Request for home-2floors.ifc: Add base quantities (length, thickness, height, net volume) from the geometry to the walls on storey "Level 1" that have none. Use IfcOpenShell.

First a look at what the model holds.

```python
import ifcopenshell
import ifcopenshell.util.element
import ifcopenshell.util.unit

model = ifcopenshell.open("home-2floors.ifc")
print(model.schema)
for unit_type in ("LENGTHUNIT", "AREAUNIT", "VOLUMEUNIT"):
    print(unit_type, ifcopenshell.util.unit.calculate_unit_scale(model, unit_type))
storey = next(s for s in model.by_type("IfcBuildingStorey") if s.Name == "Level 1")
walls = [e for e in ifcopenshell.util.element.get_decomposition(storey) if e.is_a("IfcWall")]
for e in sorted(walls, key=lambda e: e.id()):
    print(e.id(), e.is_a(), e.Name, list(ifcopenshell.util.element.get_psets(e, qtos_only=True)), sep=" | ")
```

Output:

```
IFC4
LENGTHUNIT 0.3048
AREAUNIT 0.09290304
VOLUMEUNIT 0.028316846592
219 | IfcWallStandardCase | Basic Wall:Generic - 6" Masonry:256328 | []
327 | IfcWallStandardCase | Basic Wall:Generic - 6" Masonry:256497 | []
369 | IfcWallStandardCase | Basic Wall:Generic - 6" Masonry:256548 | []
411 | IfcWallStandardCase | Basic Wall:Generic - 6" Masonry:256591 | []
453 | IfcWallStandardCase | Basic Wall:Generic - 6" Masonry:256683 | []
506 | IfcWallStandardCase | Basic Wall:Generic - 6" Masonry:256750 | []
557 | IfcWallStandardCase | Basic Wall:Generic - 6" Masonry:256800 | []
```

```python
import ifcopenshell
import ifcopenshell.api.pset
import ifcopenshell.geom
import ifcopenshell.util.element
import ifcopenshell.util.shape
import ifcopenshell.util.unit

model = ifcopenshell.open("home-2floors.ifc")
unit_scale = ifcopenshell.util.unit.calculate_unit_scale(model)
volume_scale = ifcopenshell.util.unit.calculate_unit_scale(model, "VOLUMEUNIT")
settings = ifcopenshell.geom.settings()

storey = next(s for s in model.by_type("IfcBuildingStorey") if s.Name == "Level 1")
walls = [e for e in ifcopenshell.util.element.get_decomposition(storey) if e.is_a("IfcWall")]

for e in sorted(walls, key=lambda e: e.id()):
    if ifcopenshell.util.element.get_psets(e, qtos_only=True, should_inherit=False):
        continue
    # Geometry comes back in metres, in the element's own axes.
    shape = ifcopenshell.geom.create_shape(settings, e)
    values = {
        "Length": ifcopenshell.util.shape.get_x(shape.geometry) / unit_scale,
        "Width": ifcopenshell.util.shape.get_y(shape.geometry) / unit_scale,
        "Height": ifcopenshell.util.shape.get_z(shape.geometry) / unit_scale,
        "NetVolume": ifcopenshell.util.shape.get_volume(shape.geometry) / volume_scale,
    }
    qto = ifcopenshell.api.pset.add_qto(model, product=e, name="Qto_WallBaseQuantities")
    ifcopenshell.api.pset.edit_qto(model, qto=qto, properties=values)
    print(e.id(), {k: round(v, 3) for k, v in values.items()})

model.write("home-2floors_rev.ifc")
```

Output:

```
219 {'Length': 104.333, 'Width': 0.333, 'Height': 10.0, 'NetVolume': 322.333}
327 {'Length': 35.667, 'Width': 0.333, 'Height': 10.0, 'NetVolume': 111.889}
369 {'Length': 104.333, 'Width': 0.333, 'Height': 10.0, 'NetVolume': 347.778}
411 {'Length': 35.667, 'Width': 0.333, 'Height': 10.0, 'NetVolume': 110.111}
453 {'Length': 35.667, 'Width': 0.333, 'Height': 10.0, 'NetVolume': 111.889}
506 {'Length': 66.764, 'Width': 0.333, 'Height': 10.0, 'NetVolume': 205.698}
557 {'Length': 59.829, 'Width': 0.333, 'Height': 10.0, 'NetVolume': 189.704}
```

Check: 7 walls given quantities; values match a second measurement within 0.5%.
